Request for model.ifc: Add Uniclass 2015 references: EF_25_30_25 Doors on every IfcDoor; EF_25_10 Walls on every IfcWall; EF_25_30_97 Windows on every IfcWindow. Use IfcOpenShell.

First a look at what the model holds.

```python
import ifcopenshell

model = ifcopenshell.open("model.ifc")
print(model.schema)
print("classifications:", [c.Name for c in model.by_type("IfcClassification")])
for ifc_class in ("IfcDoor", "IfcRoof", "IfcStair", "IfcWall", "IfcWindow"):
    print(ifc_class, len(model.by_type(ifc_class)))
```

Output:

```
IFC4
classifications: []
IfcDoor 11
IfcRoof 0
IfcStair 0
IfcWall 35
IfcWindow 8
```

```python
import ifcopenshell
import ifcopenshell.api.classification

model = ifcopenshell.open("model.ifc")

system = ifcopenshell.api.classification.add_classification(model, classification="Uniclass 2015")

codes = {
    "IfcDoor": ("EF_25_30_25", "Doors"),
    "IfcWall": ("EF_25_10", "Walls"),
    "IfcWindow": ("EF_25_30_97", "Windows"),
}
for ifc_class, (code, name) in codes.items():
    products = model.by_type(ifc_class)
    ifcopenshell.api.classification.add_reference(
        model, products=products, classification=system, identification=code, name=name
    )
    print(code, len(products))

model.write("model_rev.ifc")
```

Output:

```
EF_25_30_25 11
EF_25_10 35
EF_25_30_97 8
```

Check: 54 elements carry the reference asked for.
